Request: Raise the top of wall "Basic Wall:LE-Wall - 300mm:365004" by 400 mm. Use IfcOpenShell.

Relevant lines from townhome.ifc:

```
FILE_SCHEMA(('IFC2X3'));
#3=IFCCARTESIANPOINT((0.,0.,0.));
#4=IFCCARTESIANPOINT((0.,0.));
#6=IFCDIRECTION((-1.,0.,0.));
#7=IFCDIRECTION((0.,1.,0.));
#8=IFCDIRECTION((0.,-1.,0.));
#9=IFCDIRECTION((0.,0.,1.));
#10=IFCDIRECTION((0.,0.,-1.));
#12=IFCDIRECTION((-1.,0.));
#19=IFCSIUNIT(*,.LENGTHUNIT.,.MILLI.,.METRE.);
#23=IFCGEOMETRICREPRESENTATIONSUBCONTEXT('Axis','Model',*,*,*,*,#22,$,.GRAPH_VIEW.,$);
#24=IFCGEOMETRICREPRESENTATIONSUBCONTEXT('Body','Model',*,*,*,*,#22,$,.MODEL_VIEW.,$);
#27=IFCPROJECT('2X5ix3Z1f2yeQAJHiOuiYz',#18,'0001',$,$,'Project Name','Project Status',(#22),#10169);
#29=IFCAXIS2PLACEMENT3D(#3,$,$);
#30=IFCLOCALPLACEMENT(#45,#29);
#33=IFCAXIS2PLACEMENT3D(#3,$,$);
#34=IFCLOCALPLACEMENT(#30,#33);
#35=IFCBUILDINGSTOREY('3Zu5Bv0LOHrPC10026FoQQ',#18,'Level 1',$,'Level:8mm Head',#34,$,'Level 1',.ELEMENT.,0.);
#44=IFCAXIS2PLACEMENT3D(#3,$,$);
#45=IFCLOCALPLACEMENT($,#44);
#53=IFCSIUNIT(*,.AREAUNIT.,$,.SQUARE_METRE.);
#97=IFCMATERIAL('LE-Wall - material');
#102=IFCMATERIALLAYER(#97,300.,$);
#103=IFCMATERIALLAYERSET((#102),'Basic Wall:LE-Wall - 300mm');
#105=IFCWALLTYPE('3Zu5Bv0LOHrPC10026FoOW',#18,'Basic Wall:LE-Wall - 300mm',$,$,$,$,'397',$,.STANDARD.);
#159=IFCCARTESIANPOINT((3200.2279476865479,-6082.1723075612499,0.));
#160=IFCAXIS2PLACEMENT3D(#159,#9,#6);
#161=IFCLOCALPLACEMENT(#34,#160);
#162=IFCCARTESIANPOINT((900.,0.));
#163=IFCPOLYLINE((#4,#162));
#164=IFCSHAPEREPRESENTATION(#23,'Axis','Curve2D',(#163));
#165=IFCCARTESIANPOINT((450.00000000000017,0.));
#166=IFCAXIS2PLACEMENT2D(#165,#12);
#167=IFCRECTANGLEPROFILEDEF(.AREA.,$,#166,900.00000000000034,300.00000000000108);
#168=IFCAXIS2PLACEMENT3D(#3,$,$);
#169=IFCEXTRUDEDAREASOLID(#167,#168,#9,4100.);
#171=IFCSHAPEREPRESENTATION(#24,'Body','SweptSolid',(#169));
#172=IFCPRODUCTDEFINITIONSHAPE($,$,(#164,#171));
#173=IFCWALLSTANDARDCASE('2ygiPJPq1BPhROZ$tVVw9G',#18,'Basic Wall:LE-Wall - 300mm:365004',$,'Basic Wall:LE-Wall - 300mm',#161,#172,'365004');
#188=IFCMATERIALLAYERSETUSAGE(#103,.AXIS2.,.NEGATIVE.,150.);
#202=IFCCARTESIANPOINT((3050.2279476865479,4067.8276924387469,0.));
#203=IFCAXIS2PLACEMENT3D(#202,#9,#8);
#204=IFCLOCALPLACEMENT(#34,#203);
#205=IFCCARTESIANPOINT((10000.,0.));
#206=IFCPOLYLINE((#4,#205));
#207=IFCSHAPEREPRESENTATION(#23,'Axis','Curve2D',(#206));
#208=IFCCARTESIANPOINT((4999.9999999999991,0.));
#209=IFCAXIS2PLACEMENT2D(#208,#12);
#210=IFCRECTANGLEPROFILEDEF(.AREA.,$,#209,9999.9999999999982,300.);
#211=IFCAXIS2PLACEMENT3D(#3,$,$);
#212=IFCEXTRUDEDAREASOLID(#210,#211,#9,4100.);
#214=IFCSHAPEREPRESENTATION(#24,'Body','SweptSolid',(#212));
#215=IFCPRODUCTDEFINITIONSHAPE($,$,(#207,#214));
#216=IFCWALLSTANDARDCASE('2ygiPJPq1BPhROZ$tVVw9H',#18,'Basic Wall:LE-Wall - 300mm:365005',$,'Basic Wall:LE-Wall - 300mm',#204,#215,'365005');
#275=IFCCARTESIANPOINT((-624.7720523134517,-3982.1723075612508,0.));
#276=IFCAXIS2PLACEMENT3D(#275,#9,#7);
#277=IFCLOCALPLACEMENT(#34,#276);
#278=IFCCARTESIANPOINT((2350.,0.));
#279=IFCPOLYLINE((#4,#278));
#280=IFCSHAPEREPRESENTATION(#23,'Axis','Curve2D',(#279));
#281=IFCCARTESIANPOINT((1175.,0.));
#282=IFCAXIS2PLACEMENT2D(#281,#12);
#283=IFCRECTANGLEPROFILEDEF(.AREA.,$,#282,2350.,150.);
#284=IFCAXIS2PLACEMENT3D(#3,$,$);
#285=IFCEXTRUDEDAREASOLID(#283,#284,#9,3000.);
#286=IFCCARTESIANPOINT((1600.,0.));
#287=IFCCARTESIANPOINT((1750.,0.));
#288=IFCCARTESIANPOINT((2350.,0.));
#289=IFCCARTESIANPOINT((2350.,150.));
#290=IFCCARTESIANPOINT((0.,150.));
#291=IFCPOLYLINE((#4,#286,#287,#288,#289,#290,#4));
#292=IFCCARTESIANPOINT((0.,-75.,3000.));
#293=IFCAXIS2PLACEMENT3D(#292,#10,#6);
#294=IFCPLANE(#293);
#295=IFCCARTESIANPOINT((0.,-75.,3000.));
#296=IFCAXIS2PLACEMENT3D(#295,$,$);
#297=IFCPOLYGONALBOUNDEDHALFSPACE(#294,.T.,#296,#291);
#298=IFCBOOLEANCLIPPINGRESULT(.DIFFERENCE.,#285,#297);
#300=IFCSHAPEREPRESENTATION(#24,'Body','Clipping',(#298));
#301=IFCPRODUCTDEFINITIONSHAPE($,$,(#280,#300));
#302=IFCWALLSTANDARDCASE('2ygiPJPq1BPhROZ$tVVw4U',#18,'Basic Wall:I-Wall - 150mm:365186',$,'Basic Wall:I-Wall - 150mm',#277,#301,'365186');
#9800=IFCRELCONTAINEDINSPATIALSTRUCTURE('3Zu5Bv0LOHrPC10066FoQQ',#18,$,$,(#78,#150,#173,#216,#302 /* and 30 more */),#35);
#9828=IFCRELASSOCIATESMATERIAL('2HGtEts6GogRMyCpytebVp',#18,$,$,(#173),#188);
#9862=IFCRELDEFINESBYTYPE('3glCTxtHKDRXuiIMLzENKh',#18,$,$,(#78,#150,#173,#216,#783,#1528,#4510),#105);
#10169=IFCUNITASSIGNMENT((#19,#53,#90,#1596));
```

```python
import ifcopenshell
import ifcopenshell.geom
import ifcopenshell.util.representation
import ifcopenshell.util.shape

model = ifcopenshell.open("townhome.ifc")
settings = ifcopenshell.geom.settings()


def volume(element):
    """Net volume in cubic metres, openings subtracted."""
    shape = ifcopenshell.geom.create_shape(settings, element)
    return ifcopenshell.util.shape.get_volume(shape.geometry)


wall = model.by_guid("2ygiPJPq1BPhROZ$tVVw9G")
before = volume(wall)

body = ifcopenshell.util.representation.get_representation(wall, "Model", "Body")
solid = body.Items[0]
old_height = solid.Depth
solid.Depth += 400.0
after = volume(wall)

print(f"height {old_height:g} -> {solid.Depth:g}, volume {before:.3f} -> {after:.3f} m3")

model.write("townhome_v2.ifc")
```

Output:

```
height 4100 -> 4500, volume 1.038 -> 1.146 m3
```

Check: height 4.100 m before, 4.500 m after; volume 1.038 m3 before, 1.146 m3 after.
